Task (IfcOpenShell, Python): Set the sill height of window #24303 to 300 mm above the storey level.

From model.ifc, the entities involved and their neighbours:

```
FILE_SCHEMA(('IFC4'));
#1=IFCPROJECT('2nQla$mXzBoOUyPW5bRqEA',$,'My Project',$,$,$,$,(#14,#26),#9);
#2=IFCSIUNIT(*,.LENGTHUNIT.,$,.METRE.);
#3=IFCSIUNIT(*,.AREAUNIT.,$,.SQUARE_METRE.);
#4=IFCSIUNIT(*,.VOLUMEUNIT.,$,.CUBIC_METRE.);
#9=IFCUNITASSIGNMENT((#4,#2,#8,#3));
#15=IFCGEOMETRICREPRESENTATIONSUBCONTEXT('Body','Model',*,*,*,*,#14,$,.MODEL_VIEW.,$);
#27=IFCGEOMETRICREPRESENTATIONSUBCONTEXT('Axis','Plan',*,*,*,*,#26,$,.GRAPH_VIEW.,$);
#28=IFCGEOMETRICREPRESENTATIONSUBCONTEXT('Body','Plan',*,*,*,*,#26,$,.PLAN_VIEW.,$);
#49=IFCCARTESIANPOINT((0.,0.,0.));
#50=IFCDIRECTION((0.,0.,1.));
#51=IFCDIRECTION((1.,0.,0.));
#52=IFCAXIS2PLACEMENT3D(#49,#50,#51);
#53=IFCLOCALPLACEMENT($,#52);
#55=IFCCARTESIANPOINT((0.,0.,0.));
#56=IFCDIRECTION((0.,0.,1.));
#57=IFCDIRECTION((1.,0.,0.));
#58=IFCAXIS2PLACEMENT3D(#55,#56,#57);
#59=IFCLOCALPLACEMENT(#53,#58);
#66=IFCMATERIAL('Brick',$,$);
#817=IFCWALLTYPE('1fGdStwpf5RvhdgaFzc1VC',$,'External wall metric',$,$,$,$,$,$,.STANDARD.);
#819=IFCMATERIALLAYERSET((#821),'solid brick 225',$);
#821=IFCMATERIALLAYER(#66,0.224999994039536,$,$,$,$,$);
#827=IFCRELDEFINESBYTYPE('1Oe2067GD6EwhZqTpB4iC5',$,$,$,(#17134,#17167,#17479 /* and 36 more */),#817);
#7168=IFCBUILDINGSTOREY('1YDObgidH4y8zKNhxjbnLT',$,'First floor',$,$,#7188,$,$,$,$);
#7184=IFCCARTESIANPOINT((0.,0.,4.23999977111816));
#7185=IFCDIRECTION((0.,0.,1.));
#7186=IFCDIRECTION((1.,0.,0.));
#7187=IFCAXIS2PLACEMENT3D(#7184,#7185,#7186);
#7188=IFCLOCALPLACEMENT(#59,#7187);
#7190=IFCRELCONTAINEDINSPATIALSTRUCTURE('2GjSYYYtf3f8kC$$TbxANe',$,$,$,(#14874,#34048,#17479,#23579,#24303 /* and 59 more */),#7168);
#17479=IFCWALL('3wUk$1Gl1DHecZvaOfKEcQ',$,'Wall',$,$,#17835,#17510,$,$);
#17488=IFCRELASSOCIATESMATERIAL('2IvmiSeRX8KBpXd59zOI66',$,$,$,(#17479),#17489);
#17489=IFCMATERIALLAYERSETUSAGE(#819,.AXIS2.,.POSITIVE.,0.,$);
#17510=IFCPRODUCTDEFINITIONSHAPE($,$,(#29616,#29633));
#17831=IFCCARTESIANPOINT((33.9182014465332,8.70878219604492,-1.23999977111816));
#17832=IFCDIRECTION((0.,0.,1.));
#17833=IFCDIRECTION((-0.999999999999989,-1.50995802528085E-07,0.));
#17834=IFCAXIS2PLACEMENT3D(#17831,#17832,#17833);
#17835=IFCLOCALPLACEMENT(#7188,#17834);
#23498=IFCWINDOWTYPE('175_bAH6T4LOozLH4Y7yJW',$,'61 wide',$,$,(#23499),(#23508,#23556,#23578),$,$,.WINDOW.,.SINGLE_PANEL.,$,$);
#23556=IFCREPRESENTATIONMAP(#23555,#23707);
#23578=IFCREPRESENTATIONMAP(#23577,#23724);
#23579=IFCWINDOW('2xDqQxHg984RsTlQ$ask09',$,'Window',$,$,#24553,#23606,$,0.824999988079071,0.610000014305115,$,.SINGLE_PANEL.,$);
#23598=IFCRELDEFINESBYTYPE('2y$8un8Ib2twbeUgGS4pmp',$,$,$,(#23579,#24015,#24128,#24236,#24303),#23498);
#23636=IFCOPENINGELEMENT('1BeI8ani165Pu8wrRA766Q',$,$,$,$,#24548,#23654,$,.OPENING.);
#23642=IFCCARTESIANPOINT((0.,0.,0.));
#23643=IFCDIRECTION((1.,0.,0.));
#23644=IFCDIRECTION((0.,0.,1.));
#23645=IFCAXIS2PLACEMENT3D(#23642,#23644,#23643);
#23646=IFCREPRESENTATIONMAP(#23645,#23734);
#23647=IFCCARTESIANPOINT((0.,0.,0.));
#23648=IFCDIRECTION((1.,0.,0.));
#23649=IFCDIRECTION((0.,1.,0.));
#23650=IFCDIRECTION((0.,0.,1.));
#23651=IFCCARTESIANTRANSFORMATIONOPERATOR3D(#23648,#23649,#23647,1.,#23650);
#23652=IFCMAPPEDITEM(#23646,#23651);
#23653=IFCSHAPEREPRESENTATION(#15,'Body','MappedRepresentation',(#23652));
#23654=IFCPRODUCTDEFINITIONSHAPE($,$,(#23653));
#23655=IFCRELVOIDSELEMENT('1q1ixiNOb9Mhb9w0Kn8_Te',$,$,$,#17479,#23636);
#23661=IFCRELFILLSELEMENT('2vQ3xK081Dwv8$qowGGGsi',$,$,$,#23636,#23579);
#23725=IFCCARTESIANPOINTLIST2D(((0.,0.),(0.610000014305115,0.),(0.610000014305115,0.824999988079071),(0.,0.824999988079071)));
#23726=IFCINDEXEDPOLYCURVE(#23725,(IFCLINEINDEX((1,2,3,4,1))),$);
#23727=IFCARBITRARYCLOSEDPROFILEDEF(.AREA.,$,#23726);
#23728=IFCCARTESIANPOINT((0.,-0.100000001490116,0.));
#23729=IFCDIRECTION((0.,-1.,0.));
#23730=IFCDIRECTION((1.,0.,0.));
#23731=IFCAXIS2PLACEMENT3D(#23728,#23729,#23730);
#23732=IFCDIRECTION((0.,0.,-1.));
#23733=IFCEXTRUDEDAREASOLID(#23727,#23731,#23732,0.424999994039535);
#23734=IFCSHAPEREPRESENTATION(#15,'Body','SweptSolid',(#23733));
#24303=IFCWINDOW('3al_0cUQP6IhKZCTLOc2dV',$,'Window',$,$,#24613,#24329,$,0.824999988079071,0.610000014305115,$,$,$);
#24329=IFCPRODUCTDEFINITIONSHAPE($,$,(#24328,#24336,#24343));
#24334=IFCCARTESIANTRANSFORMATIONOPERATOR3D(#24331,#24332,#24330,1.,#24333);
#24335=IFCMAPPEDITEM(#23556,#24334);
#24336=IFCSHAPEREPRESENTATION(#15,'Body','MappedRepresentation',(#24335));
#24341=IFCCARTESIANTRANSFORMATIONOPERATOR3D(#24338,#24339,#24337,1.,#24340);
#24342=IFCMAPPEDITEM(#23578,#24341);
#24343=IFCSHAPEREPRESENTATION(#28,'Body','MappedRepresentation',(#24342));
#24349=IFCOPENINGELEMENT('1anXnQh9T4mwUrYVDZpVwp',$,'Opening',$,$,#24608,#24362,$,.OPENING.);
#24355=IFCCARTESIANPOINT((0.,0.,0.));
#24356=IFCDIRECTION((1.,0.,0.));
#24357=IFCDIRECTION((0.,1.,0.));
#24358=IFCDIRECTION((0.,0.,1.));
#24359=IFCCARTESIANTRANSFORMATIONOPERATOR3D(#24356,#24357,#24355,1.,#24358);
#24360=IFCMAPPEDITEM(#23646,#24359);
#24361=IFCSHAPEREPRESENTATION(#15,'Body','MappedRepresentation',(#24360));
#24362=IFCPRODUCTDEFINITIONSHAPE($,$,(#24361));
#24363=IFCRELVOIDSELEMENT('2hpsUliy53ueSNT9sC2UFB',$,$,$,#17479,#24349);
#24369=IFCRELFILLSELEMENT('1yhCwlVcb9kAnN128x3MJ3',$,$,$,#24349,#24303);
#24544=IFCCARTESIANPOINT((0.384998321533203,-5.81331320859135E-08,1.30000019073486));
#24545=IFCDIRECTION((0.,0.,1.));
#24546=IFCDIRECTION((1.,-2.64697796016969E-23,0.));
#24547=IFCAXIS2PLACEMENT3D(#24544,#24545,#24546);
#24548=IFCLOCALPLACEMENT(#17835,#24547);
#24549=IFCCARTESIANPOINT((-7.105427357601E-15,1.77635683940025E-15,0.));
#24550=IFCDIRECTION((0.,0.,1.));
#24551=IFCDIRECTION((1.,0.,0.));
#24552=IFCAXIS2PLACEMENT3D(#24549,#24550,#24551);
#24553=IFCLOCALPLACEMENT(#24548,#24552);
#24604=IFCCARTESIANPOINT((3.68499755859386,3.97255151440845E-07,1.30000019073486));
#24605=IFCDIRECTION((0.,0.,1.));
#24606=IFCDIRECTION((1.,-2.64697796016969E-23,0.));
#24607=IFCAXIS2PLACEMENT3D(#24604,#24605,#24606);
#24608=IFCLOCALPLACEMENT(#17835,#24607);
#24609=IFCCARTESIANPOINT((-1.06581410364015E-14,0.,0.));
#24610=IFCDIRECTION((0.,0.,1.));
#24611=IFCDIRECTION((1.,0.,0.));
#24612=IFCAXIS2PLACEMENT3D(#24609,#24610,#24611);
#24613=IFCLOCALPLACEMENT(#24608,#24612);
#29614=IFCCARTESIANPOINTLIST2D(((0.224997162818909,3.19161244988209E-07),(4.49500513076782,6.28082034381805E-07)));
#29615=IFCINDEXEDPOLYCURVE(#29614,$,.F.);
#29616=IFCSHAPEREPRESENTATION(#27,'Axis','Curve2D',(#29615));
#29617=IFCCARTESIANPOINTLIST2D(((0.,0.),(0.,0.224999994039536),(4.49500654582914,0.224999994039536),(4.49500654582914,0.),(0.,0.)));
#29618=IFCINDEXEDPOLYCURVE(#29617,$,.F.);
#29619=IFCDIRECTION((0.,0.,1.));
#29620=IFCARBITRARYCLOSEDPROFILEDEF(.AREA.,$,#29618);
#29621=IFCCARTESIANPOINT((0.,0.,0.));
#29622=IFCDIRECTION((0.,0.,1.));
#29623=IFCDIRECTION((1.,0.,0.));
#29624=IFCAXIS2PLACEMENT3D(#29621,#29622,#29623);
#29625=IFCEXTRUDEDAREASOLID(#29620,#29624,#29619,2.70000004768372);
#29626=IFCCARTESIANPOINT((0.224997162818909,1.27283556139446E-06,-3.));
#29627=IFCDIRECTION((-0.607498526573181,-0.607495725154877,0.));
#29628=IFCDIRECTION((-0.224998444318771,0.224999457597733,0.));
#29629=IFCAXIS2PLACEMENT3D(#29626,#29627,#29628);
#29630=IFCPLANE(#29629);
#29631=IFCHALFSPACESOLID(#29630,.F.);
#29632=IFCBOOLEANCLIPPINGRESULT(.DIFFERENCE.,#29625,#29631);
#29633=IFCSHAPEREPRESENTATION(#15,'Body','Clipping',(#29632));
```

```python
import numpy as np
import ifcopenshell
import ifcopenshell.api.geometry
import ifcopenshell.geom
import ifcopenshell.util.element
import ifcopenshell.util.placement
import ifcopenshell.util.shape
import ifcopenshell.util.unit

model = ifcopenshell.open("model.ifc")
unit_scale = ifcopenshell.util.unit.calculate_unit_scale(model)

window = model.by_guid("3al_0cUQP6IhKZCTLOc2dV")
opening = window.FillsVoids[0].RelatingOpeningElement
storey = ifcopenshell.util.element.get_container(window, ifc_class="IfcBuildingStorey")
level = ifcopenshell.util.placement.get_local_placement(storey.ObjectPlacement)[2, 3]

# The opening's origin need not be at the sill, so measure its lowest point.
shape = ifcopenshell.geom.create_shape(ifcopenshell.geom.settings(), opening)
bottom = ifcopenshell.util.shape.get_shape_bottom_elevation(shape, shape.geometry) / unit_scale
dz = level + 0.3 - bottom

shift = np.array([0.0, 0.0, dz])
# The window is placed relative to its opening, so it follows when the opening moves.
matrix = ifcopenshell.util.placement.get_local_placement(opening.ObjectPlacement)
matrix[:3, 3] += shift
ifcopenshell.api.geometry.edit_object_placement(
    model, product=opening, matrix=matrix, is_si=False, should_transform_children=True
)

print(f"moved by {dz * unit_scale:+.3f} m")

model.write("model_updated.ifc")
```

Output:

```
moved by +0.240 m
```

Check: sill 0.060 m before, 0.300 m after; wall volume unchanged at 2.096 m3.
